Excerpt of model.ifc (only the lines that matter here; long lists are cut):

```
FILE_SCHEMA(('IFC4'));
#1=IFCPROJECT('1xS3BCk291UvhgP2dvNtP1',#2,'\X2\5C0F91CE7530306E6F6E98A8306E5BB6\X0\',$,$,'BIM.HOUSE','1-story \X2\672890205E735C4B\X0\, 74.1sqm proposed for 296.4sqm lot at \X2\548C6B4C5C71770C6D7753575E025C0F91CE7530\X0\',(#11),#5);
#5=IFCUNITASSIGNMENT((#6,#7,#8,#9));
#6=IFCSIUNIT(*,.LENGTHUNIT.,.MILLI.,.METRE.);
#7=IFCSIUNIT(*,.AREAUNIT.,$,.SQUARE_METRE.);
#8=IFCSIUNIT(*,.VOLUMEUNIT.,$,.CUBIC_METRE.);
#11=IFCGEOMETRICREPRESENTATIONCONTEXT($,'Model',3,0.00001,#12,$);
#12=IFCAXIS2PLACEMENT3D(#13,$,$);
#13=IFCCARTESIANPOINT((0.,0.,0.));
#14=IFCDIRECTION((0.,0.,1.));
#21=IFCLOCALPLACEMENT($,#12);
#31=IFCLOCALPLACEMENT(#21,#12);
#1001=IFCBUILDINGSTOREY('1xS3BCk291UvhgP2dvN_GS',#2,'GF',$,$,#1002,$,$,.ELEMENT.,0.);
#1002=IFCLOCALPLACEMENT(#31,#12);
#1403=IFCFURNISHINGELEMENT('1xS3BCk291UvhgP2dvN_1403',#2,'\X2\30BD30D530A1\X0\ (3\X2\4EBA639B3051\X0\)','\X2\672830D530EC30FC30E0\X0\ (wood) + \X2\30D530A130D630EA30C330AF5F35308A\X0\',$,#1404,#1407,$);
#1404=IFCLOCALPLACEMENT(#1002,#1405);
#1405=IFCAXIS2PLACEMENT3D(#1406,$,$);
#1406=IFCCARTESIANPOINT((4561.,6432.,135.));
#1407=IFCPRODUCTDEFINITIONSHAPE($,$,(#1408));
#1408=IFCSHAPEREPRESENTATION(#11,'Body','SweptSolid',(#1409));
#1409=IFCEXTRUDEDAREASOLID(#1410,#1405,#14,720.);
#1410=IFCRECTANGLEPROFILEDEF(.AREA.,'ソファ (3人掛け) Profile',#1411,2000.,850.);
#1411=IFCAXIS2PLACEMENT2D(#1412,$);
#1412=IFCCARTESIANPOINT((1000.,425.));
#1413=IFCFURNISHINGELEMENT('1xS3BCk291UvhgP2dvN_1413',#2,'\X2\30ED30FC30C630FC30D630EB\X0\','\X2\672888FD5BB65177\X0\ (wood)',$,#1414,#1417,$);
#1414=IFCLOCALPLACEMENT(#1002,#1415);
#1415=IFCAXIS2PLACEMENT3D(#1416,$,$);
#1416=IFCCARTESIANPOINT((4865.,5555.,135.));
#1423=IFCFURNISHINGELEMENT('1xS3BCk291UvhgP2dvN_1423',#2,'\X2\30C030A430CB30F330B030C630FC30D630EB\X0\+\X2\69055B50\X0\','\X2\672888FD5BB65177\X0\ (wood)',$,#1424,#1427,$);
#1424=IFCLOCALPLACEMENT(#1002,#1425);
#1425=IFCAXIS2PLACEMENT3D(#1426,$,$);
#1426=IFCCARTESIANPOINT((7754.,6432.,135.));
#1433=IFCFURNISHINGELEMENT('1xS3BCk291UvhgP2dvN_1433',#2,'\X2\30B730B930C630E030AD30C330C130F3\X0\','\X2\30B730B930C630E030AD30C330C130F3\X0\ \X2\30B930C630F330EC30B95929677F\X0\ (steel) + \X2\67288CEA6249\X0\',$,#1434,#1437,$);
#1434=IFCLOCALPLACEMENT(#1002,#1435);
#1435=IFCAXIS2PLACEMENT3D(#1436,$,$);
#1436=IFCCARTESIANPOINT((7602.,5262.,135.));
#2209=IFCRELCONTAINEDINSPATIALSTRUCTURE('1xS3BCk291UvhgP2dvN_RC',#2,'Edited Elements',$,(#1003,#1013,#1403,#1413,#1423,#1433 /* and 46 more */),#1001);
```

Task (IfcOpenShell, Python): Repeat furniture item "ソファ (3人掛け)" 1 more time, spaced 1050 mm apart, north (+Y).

```python
import numpy as np
import ifcopenshell
import ifcopenshell.api.geometry
import ifcopenshell.api.root
import ifcopenshell.util.element
import ifcopenshell.util.placement
import ifcopenshell.util.unit

model = ifcopenshell.open("model.ifc")
unit_scale = ifcopenshell.util.unit.calculate_unit_scale(model)


def reuse_history(source, copy):
    """copy_class also copies each property set's owner history, people and application; keep the originals."""
    for rel in copy.IsDefinedBy:
        if rel.is_a("IfcRelDefinesByProperties") and (history := rel.RelatingPropertyDefinition.OwnerHistory):
            rel.RelatingPropertyDefinition.OwnerHistory = source.OwnerHistory
            ifcopenshell.util.element.remove_deep2(model, history)


source = model.by_guid("1xS3BCk291UvhgP2dvN_1403")
base = ifcopenshell.util.placement.get_local_placement(source.ObjectPlacement)
step = np.array([0.0, 1.0, 0.0]) * 1.05 / unit_scale

for i in range(1, 2):
    copy = ifcopenshell.api.root.copy_class(model, product=source)
    copy.Representation = ifcopenshell.util.element.copy_deep(
        model, source.Representation, exclude=["IfcGeometricRepresentationContext", "IfcRepresentationMap"]
    )
    reuse_history(source, copy)
    matrix = base.copy()
    matrix[:3, 3] += i * step
    print("added at", matrix[:3, 3].round(3) + 0.0)
    ifcopenshell.api.geometry.edit_object_placement(model, product=copy, matrix=matrix, is_si=False)

model.write("model-out.ifc")
```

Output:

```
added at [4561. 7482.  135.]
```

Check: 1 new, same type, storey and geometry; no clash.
